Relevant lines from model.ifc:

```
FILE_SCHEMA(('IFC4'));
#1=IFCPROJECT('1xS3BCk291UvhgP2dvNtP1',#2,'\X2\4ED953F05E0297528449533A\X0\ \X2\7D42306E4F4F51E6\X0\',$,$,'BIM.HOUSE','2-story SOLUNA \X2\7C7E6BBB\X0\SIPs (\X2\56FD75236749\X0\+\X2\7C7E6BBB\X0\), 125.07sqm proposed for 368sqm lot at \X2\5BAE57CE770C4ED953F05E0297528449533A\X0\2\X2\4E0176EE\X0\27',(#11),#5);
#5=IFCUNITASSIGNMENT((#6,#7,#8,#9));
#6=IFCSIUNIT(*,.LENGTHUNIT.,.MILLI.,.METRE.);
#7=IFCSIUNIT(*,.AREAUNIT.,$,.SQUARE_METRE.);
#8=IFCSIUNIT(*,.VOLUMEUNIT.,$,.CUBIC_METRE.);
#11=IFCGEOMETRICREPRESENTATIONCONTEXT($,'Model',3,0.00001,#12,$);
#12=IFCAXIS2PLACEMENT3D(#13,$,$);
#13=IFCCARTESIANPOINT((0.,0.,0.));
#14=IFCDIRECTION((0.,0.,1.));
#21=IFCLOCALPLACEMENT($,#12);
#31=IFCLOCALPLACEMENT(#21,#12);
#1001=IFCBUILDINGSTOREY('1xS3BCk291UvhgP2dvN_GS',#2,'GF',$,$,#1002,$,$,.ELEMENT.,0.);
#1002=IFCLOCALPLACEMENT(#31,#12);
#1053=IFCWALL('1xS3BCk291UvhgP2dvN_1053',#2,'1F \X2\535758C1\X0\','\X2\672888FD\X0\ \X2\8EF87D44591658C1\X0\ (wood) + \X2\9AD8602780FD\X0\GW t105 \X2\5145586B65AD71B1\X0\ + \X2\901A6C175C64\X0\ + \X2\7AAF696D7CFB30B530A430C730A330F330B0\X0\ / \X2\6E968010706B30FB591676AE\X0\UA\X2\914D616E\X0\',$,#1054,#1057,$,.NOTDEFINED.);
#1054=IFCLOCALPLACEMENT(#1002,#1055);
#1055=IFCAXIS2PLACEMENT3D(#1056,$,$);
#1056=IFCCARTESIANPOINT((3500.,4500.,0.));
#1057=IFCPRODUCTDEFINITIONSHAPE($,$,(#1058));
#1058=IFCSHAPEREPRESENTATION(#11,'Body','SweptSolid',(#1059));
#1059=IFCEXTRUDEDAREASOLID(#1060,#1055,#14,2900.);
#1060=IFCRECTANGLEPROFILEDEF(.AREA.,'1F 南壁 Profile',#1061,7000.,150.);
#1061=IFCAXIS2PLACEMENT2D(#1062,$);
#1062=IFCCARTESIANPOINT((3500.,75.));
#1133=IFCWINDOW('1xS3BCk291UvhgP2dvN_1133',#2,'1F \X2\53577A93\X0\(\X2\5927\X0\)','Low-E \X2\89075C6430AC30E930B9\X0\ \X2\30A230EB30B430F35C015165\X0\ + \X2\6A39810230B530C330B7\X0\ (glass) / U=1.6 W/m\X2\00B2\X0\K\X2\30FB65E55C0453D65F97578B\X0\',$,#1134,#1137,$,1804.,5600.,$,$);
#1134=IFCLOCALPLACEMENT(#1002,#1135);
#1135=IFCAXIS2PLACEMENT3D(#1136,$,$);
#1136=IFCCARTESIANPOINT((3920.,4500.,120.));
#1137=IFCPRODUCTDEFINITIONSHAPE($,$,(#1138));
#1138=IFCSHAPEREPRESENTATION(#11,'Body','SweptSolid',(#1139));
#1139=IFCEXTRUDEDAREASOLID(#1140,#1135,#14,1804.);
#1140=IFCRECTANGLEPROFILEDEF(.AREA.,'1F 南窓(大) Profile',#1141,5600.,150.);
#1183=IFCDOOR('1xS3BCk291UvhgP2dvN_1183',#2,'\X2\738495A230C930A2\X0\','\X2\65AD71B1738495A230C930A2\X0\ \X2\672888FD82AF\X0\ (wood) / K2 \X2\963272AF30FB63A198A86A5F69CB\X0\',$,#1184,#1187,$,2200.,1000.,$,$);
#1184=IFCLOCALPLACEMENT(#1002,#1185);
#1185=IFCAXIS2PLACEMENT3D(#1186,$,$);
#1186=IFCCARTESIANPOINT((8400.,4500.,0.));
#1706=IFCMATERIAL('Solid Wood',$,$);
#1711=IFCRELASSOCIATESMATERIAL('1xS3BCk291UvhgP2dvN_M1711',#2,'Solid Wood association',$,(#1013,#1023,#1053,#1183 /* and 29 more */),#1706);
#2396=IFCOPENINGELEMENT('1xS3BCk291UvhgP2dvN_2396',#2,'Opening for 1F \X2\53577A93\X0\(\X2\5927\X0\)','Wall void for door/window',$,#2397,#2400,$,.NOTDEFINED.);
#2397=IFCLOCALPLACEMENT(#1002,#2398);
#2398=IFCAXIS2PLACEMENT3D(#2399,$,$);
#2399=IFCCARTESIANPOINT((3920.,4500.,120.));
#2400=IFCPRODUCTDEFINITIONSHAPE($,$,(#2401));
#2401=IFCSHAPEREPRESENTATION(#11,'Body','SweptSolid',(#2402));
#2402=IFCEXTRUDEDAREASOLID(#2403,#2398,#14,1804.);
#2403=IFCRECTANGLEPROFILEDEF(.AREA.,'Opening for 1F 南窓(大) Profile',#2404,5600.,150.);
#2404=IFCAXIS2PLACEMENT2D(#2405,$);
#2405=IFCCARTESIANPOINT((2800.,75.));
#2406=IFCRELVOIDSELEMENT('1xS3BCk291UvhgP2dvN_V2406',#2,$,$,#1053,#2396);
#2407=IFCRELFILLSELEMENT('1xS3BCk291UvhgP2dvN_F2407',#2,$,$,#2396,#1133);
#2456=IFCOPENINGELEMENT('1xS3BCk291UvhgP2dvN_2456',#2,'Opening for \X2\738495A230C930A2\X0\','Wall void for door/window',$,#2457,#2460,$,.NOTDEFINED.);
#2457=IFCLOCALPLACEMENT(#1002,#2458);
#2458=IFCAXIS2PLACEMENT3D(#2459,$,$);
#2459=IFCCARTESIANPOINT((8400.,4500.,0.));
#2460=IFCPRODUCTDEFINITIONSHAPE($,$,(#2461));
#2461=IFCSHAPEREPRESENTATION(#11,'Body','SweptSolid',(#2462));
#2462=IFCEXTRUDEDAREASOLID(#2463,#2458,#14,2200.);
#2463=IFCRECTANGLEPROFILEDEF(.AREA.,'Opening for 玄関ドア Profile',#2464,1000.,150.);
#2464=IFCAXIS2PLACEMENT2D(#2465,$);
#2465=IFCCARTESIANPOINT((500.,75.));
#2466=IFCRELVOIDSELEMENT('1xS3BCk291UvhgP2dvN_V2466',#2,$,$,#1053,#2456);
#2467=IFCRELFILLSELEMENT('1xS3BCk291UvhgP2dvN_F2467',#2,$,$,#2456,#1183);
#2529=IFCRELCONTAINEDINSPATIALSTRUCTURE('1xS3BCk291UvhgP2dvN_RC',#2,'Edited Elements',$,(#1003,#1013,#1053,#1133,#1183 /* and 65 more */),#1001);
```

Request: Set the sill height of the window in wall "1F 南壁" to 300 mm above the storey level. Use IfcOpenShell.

```python
import numpy as np
import ifcopenshell
import ifcopenshell.api.geometry
import ifcopenshell.geom
import ifcopenshell.util.element
import ifcopenshell.util.placement
import ifcopenshell.util.shape
import ifcopenshell.util.unit

model = ifcopenshell.open("model.ifc")
unit_scale = ifcopenshell.util.unit.calculate_unit_scale(model)

window = model.by_guid("1xS3BCk291UvhgP2dvN_1133")
opening = window.FillsVoids[0].RelatingOpeningElement
storey = ifcopenshell.util.element.get_container(window, ifc_class="IfcBuildingStorey")
level = ifcopenshell.util.placement.get_local_placement(storey.ObjectPlacement)[2, 3]

# The opening's origin need not be at the sill, so measure its lowest point.
shape = ifcopenshell.geom.create_shape(ifcopenshell.geom.settings(), opening)
bottom = ifcopenshell.util.shape.get_shape_bottom_elevation(shape, shape.geometry) / unit_scale
dz = level + 0.3 / unit_scale - bottom

shift = np.array([0.0, 0.0, dz])
# The window is not placed relative to its opening, so move both.
for product in (opening, window):
    matrix = ifcopenshell.util.placement.get_local_placement(product.ObjectPlacement)
    matrix[:3, 3] += shift
    ifcopenshell.api.geometry.edit_object_placement(model, product=product, matrix=matrix, is_si=False)

print(f"moved by {dz * unit_scale:+.3f} m")

model.write("model_v2.ifc")
```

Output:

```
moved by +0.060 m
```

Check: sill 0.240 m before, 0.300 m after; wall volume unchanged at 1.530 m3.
